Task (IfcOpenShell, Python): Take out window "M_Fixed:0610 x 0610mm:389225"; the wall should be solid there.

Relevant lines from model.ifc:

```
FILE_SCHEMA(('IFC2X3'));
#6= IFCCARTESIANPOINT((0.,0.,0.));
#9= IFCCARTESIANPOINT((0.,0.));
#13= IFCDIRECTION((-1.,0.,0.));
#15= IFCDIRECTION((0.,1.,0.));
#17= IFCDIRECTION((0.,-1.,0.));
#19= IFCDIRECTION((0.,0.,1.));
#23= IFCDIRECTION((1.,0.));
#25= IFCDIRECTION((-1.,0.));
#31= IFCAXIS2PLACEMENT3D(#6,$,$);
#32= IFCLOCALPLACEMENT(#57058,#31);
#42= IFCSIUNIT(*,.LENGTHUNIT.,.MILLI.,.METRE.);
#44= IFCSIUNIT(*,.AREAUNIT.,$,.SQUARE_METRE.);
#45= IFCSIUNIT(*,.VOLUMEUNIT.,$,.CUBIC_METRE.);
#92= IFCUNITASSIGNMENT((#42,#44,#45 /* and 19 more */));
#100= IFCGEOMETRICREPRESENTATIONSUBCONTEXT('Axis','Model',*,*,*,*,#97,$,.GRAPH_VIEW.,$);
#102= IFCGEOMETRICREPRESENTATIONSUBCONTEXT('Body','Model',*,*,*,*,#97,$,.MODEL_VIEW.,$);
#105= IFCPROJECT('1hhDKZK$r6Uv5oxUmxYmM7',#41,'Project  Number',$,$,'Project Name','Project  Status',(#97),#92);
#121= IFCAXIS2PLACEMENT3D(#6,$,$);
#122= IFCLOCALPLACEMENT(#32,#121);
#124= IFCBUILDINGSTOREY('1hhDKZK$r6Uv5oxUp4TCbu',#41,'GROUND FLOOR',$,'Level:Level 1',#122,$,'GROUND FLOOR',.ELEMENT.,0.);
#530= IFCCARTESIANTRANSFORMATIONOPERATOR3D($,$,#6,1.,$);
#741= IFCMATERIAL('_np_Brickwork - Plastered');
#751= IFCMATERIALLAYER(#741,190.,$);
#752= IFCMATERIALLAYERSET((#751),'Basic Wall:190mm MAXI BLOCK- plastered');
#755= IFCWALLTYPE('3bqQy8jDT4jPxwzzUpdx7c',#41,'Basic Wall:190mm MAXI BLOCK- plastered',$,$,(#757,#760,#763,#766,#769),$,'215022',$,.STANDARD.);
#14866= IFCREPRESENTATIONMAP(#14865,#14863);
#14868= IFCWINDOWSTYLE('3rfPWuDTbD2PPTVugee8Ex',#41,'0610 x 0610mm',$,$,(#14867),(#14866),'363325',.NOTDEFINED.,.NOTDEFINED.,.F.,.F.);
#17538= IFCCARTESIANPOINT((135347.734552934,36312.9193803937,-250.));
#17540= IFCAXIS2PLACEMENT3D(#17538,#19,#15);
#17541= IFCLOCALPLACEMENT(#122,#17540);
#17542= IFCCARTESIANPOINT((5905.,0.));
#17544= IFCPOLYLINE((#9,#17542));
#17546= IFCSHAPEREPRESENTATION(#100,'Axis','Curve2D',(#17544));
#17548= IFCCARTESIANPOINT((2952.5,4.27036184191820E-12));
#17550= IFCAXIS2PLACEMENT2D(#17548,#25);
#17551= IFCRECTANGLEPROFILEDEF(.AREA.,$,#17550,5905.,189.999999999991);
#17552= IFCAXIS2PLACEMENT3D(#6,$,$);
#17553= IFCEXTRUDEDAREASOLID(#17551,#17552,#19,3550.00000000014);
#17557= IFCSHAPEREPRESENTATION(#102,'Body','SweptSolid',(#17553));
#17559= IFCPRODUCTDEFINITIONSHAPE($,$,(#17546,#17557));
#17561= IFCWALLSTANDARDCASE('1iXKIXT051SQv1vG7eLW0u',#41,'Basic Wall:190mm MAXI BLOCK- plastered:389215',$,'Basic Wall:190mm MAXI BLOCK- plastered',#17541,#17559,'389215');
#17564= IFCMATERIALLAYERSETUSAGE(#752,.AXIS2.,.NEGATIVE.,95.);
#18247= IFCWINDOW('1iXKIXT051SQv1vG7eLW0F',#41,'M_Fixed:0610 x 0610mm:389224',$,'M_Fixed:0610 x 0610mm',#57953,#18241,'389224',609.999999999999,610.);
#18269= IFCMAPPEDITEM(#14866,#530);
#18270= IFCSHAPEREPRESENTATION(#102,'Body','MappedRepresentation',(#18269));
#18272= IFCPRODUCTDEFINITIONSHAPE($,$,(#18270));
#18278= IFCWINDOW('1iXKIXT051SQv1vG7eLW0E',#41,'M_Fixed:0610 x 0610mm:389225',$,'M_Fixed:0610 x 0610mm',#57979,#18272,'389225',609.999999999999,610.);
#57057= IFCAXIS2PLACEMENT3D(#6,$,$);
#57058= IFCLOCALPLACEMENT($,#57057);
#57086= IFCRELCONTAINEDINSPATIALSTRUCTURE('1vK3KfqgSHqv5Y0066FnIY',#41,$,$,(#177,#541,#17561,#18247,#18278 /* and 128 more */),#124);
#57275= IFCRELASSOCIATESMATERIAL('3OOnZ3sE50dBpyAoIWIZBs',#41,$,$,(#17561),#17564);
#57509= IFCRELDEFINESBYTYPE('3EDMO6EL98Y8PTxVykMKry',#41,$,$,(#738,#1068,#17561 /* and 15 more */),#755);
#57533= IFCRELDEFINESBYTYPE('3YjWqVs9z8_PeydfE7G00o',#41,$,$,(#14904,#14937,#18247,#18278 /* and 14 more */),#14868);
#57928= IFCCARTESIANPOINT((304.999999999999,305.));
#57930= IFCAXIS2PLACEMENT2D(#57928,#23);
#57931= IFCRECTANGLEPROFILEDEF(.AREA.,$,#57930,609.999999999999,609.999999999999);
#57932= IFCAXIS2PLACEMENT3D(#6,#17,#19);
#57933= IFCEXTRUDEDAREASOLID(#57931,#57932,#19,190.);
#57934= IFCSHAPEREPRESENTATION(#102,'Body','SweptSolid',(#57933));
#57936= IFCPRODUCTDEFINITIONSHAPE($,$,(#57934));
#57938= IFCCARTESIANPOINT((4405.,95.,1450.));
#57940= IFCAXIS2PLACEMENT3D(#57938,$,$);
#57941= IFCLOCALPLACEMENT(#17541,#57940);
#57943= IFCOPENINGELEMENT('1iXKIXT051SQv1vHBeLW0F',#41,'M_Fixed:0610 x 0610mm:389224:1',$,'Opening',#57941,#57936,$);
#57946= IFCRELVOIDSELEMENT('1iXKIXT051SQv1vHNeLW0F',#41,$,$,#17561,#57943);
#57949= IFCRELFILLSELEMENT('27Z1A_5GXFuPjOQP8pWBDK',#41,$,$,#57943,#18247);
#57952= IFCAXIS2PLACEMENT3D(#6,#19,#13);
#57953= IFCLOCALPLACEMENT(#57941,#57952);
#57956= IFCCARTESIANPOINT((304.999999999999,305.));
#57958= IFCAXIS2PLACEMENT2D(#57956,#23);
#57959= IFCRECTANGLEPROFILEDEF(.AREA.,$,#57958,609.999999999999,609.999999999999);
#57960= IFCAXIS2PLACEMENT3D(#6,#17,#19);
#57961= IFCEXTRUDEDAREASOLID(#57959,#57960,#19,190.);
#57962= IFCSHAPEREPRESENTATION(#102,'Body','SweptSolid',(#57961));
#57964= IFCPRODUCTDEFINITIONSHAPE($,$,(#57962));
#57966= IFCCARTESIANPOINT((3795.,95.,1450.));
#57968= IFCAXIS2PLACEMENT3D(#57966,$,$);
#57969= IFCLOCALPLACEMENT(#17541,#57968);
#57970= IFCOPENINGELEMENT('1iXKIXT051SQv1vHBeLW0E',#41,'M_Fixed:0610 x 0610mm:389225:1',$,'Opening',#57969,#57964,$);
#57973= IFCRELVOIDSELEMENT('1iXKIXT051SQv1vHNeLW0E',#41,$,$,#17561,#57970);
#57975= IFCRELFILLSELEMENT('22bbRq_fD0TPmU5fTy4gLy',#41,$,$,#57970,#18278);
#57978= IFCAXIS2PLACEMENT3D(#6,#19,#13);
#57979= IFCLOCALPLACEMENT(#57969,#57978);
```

```python
import ifcopenshell
import ifcopenshell.api.feature
import ifcopenshell.api.root
import ifcopenshell.geom
import ifcopenshell.util.shape

model = ifcopenshell.open("model.ifc")
settings = ifcopenshell.geom.settings()


def volume(element):
    """Net volume in cubic metres, openings subtracted."""
    shape = ifcopenshell.geom.create_shape(settings, element)
    return ifcopenshell.util.shape.get_volume(shape.geometry)


window = model.by_guid("1iXKIXT051SQv1vG7eLW0E")
opening = window.FillsVoids[0].RelatingOpeningElement
wall = opening.VoidsElements[0].RelatingBuildingElement
before = volume(wall)

ifcopenshell.api.root.remove_product(model, product=window)
ifcopenshell.api.feature.remove_feature(model, feature=opening)

after = volume(wall)

print(f"wall volume {before:.3f} -> {after:.3f} m3")

model.write("model_rev.ifc")
```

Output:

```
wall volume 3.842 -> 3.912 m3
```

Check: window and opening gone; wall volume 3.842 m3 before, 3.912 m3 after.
